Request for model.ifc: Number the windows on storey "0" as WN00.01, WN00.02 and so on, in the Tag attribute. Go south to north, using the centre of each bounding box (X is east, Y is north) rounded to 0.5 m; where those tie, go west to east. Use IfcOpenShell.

First a look at what the model holds.

```python
import ifcopenshell
import ifcopenshell.util.element
import ifcopenshell.util.placement

model = ifcopenshell.open("model.ifc")
print(model.schema)
storey = next(s for s in model.by_type("IfcBuildingStorey") if s.Name == "0")
windows = [e for e in ifcopenshell.util.element.get_decomposition(storey) if e.is_a("IfcWindow")]
for e in sorted(windows, key=lambda e: e.id()):
    origin = ifcopenshell.util.placement.get_local_placement(e.ObjectPlacement)[:3, 3]
    print(e.id(), e.Tag, e.Name, origin.round(2) + 0.0, sep=" | ")
```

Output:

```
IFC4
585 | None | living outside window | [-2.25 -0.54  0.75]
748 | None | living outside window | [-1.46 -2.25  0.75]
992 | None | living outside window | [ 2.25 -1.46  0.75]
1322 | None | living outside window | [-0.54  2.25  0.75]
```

```python
import ifcopenshell
import ifcopenshell.geom
import ifcopenshell.util.element
import ifcopenshell.util.shape

model = ifcopenshell.open("model.ifc")
settings = ifcopenshell.geom.settings()
settings.set("use-world-coords", True)


def centre(element):
    shape = ifcopenshell.geom.create_shape(settings, element)
    return ifcopenshell.util.shape.get_bbox_centroid(shape.geometry)


storey = next(s for s in model.by_type("IfcBuildingStorey") if s.Name == "0")
windows = [e for e in ifcopenshell.util.element.get_decomposition(storey) if e.is_a("IfcWindow")]

# Insertion points can sit at a corner or the storey origin, so sort by the geometry (in metres).
centres = {e: centre(e) for e in windows}
windows.sort(key=lambda e: (round(centres[e][1] / 0.5), centres[e][0]))

for i, e in enumerate(windows, start=1):
    number = f"WN00.{i:02d}"
    e.Tag = number
    print(e.id(), number)

model.write("model_edited.ifc")
```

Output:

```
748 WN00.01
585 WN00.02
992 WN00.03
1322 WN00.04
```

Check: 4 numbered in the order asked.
